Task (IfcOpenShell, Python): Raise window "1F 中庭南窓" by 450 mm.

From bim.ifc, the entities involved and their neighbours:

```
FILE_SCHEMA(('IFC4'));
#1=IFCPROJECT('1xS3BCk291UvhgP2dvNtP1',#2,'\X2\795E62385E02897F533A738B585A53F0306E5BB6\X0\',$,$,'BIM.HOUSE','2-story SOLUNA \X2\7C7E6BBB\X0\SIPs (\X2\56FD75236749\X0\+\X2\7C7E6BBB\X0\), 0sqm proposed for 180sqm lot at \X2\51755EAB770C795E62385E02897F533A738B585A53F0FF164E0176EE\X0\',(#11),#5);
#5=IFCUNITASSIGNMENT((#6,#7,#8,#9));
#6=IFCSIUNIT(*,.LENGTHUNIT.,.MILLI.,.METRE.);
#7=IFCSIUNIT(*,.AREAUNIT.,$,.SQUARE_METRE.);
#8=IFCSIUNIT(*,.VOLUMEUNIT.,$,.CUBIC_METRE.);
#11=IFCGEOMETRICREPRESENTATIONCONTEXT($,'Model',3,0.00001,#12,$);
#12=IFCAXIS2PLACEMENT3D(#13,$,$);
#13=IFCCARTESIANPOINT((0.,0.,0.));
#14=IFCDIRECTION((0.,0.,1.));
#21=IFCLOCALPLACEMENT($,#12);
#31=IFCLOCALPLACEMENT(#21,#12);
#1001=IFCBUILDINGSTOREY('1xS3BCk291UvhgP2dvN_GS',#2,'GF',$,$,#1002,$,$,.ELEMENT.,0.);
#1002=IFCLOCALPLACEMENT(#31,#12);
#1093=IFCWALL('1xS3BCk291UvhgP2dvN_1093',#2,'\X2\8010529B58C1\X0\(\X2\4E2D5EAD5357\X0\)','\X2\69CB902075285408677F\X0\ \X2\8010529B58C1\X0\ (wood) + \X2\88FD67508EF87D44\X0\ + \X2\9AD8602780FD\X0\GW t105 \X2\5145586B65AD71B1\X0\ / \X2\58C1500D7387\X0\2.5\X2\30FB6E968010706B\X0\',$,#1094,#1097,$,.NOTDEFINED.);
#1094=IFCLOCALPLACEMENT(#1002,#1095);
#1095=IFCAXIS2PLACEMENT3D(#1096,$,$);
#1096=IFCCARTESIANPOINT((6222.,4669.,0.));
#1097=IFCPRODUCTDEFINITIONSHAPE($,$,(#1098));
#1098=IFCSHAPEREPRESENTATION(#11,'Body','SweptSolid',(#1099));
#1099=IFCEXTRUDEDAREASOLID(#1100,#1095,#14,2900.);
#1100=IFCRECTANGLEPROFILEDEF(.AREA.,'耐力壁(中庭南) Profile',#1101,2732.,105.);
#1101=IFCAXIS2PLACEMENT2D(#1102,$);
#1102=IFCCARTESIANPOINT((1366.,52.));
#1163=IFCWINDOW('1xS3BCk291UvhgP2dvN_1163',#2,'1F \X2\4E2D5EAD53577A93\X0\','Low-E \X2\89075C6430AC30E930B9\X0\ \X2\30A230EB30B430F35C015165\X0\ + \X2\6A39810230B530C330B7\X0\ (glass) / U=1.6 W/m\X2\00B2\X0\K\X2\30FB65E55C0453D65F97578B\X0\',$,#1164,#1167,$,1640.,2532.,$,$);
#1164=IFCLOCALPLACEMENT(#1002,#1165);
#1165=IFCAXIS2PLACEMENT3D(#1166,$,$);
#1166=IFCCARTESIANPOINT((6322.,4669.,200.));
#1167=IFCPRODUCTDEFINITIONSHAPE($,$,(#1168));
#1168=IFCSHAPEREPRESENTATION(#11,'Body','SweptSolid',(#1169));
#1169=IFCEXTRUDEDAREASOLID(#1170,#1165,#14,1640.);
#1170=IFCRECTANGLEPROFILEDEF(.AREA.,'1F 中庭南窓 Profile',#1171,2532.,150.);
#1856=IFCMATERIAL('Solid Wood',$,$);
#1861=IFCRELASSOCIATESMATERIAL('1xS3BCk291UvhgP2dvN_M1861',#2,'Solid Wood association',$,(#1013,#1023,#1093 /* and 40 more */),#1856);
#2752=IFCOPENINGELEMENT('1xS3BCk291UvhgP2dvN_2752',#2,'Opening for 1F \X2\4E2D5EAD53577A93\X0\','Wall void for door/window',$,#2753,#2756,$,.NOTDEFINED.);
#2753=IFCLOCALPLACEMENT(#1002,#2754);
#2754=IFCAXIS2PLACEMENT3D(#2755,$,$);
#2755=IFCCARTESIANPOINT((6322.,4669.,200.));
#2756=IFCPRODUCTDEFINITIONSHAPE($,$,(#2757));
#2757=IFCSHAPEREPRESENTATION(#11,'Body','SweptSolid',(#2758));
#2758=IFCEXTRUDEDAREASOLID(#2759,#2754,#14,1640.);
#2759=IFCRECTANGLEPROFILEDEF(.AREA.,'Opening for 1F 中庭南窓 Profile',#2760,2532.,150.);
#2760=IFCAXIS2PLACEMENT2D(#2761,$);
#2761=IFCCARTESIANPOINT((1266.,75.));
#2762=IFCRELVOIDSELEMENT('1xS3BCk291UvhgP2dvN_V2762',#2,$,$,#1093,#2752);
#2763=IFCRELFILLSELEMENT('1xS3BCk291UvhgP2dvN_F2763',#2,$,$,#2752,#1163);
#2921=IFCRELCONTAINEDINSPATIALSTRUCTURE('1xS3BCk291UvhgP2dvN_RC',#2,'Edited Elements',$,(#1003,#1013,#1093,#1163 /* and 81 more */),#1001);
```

```python
import numpy as np
import ifcopenshell
import ifcopenshell.api.geometry
import ifcopenshell.util.placement
import ifcopenshell.util.unit

model = ifcopenshell.open("bim.ifc")
unit_scale = ifcopenshell.util.unit.calculate_unit_scale(model)

window = model.by_guid("1xS3BCk291UvhgP2dvN_1163")
opening = window.FillsVoids[0].RelatingOpeningElement
dz = 0.45 / unit_scale

shift = np.array([0.0, 0.0, dz])
# The window is not placed relative to its opening, so move both.
for product in (opening, window):
    matrix = ifcopenshell.util.placement.get_local_placement(product.ObjectPlacement)
    matrix[:3, 3] += shift
    ifcopenshell.api.geometry.edit_object_placement(model, product=product, matrix=matrix, is_si=False)

print(f"moved by {dz * unit_scale:+.3f} m")

model.write("bim_updated.ifc")
```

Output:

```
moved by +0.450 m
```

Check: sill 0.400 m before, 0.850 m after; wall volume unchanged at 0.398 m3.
